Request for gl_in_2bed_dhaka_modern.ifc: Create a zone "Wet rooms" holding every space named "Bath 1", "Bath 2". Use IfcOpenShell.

First a look at what the model holds.

```python
import ifcopenshell

model = ifcopenshell.open("gl_in_2bed_dhaka_modern.ifc")
print(model.schema)
seen = {}
for space in model.by_type("IfcSpace"):
    seen[space.LongName] = seen.get(space.LongName, 0) + 1
for name, count in sorted(seen.items(), key=str):
    print(count, "x", name)
print("zones:", [z.Name for z in model.by_type("IfcZone")][:20])
```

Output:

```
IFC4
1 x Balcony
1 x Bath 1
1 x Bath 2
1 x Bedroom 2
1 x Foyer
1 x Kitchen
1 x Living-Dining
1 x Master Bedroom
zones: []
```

```python
import ifcopenshell
import ifcopenshell.api.group
import ifcopenshell.api.root

model = ifcopenshell.open("gl_in_2bed_dhaka_modern.ifc")

names = {"Bath 1", "Bath 2"}
spaces = [s for s in model.by_type("IfcSpace") if s.LongName in names]

zone = ifcopenshell.api.root.create_entity(model, ifc_class="IfcZone", name="Wet rooms")
ifcopenshell.api.group.assign_group(model, products=spaces, group=zone)
print(len(spaces), "spaces in", zone.Name)

model.write("gl_in_2bed_dhaka_modern-out.ifc")
```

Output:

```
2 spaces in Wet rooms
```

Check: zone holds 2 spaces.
